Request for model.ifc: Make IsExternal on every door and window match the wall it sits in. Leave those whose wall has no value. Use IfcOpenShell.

First a look at what the model holds.

```python
import ifcopenshell
import ifcopenshell.util.element

model = ifcopenshell.open("model.ifc")
print(model.schema)
seen = {}
for e in model.by_type("IfcDoor") + model.by_type("IfcWindow"):
    if not e.FillsVoids:
        continue
    host = e.FillsVoids[0].RelatingOpeningElement.VoidsElements[0].RelatingBuildingElement
    own = ifcopenshell.util.element.get_pset(e, f"Pset_{e.is_a()[3:].removesuffix('StandardCase')}Common", "IsExternal")
    wall = ifcopenshell.util.element.get_pset(host, "Pset_WallCommon", "IsExternal")
    seen[e.is_a(), own, wall] = seen.get((e.is_a(), own, wall), 0) + 1
for (cls, own, wall), count in sorted(seen.items(), key=str):
    print(count, cls, "IsExternal:", own, "| host wall:", wall)
```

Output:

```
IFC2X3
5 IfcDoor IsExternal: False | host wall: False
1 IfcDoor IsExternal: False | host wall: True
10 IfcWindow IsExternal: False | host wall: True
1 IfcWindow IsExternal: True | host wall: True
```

```python
import ifcopenshell
import ifcopenshell.api.pset
import ifcopenshell.util.element

model = ifcopenshell.open("model.ifc")

count = 0
for ifc_class, pset_name in (("IfcDoor", "Pset_DoorCommon"), ("IfcWindow", "Pset_WindowCommon")):
    for e in model.by_type(ifc_class):
        if not e.FillsVoids:
            continue
        host = e.FillsVoids[0].RelatingOpeningElement.VoidsElements[0].RelatingBuildingElement
        external = ifcopenshell.util.element.get_pset(host, "Pset_WallCommon", "IsExternal")
        if external is None or ifcopenshell.util.element.get_pset(e, pset_name, "IsExternal") == external:
            continue
        pset = ifcopenshell.api.pset.add_pset(model, product=e, name=pset_name)
        ifcopenshell.api.pset.edit_pset(model, pset=pset, properties={"IsExternal": external})
        count += 1

print(count, "updated")

model.write("model_v2.ifc")
```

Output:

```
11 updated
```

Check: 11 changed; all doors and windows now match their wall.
